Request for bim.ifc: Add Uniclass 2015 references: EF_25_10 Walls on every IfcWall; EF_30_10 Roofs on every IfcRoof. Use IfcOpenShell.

First a look at what the model holds.

```python
import ifcopenshell

model = ifcopenshell.open("bim.ifc")
print(model.schema)
print("classifications:", [c.Name for c in model.by_type("IfcClassification")])
for ifc_class in ("IfcDoor", "IfcRoof", "IfcStair", "IfcWall", "IfcWindow"):
    print(ifc_class, len(model.by_type(ifc_class)))
```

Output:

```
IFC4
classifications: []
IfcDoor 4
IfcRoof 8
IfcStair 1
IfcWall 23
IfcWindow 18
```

```python
import ifcopenshell
import ifcopenshell.api.classification

model = ifcopenshell.open("bim.ifc")

system = ifcopenshell.api.classification.add_classification(model, classification="Uniclass 2015")

codes = {
    "IfcWall": ("EF_25_10", "Walls"),
    "IfcRoof": ("EF_30_10", "Roofs"),
}
for ifc_class, (code, name) in codes.items():
    products = model.by_type(ifc_class)
    ifcopenshell.api.classification.add_reference(
        model, products=products, classification=system, identification=code, name=name
    )
    print(code, len(products))

model.write("bim-out.ifc")
```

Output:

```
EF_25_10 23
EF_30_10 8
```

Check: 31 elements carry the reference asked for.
